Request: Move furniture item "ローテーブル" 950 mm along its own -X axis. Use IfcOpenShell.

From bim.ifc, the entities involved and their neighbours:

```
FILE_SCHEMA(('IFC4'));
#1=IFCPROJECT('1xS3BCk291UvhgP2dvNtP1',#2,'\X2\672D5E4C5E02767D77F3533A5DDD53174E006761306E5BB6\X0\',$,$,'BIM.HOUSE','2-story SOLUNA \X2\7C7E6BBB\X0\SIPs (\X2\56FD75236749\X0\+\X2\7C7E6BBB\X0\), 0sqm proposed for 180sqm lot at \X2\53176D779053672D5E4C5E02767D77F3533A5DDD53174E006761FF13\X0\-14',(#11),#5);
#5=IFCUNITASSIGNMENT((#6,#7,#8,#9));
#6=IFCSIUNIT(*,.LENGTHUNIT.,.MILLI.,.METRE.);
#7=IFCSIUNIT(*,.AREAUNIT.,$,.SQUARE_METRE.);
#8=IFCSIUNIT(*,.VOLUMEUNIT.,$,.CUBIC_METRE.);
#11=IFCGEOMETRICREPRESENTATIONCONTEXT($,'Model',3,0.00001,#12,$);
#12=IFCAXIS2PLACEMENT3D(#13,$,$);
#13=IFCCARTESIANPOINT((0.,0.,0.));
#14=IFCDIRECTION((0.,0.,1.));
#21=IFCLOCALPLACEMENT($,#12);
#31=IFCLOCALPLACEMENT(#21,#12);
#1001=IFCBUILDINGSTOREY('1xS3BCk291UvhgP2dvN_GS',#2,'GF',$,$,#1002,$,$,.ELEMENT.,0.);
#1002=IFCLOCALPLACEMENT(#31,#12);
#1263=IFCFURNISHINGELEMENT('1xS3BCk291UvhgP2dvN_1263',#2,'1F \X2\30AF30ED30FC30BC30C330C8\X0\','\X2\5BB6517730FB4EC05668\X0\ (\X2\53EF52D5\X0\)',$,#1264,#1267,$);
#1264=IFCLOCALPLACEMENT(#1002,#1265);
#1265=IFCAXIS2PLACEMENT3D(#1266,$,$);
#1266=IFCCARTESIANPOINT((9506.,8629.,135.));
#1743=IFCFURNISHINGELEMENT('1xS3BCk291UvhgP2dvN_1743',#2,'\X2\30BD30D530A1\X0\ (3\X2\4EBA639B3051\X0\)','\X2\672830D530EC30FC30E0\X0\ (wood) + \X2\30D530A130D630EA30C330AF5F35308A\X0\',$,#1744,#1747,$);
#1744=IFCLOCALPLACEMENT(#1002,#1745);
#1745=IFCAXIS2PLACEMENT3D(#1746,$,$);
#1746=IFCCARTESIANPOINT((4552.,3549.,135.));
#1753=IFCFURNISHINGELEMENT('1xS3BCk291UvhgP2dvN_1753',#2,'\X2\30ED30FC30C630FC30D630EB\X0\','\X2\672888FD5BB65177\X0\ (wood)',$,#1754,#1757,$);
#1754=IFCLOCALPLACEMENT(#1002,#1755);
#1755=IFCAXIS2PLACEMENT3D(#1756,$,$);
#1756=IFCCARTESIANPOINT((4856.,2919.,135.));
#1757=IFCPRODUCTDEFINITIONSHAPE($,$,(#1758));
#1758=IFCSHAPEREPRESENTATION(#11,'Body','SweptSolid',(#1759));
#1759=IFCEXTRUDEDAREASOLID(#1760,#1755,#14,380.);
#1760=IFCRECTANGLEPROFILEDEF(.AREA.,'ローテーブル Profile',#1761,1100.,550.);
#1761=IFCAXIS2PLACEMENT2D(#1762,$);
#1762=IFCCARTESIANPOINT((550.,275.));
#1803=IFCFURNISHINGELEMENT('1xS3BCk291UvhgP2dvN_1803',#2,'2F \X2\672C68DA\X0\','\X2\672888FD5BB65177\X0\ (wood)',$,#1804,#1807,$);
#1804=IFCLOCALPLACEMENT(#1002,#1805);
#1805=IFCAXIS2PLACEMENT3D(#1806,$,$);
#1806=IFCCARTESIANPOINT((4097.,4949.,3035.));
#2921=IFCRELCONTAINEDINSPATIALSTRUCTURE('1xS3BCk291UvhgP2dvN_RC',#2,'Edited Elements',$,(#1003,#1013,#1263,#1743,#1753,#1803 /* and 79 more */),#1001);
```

```python
import ifcopenshell
import ifcopenshell.api.geometry
import ifcopenshell.util.placement

model = ifcopenshell.open("bim.ifc")

item = model.by_guid("1xS3BCk291UvhgP2dvN_1753")
matrix = ifcopenshell.util.placement.get_local_placement(item.ObjectPlacement)
matrix[:3, 3] -= matrix[:3, 0] * 950.0
ifcopenshell.api.geometry.edit_object_placement(model, product=item, matrix=matrix, is_si=False)

print(ifcopenshell.util.placement.get_local_placement(item.ObjectPlacement).round(3) + 0.0)

model.write("bim_rev.ifc")
```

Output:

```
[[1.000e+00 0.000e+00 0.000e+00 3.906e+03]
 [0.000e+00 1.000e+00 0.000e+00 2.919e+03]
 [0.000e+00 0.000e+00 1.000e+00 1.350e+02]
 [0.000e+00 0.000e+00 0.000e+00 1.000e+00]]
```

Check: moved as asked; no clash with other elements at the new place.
